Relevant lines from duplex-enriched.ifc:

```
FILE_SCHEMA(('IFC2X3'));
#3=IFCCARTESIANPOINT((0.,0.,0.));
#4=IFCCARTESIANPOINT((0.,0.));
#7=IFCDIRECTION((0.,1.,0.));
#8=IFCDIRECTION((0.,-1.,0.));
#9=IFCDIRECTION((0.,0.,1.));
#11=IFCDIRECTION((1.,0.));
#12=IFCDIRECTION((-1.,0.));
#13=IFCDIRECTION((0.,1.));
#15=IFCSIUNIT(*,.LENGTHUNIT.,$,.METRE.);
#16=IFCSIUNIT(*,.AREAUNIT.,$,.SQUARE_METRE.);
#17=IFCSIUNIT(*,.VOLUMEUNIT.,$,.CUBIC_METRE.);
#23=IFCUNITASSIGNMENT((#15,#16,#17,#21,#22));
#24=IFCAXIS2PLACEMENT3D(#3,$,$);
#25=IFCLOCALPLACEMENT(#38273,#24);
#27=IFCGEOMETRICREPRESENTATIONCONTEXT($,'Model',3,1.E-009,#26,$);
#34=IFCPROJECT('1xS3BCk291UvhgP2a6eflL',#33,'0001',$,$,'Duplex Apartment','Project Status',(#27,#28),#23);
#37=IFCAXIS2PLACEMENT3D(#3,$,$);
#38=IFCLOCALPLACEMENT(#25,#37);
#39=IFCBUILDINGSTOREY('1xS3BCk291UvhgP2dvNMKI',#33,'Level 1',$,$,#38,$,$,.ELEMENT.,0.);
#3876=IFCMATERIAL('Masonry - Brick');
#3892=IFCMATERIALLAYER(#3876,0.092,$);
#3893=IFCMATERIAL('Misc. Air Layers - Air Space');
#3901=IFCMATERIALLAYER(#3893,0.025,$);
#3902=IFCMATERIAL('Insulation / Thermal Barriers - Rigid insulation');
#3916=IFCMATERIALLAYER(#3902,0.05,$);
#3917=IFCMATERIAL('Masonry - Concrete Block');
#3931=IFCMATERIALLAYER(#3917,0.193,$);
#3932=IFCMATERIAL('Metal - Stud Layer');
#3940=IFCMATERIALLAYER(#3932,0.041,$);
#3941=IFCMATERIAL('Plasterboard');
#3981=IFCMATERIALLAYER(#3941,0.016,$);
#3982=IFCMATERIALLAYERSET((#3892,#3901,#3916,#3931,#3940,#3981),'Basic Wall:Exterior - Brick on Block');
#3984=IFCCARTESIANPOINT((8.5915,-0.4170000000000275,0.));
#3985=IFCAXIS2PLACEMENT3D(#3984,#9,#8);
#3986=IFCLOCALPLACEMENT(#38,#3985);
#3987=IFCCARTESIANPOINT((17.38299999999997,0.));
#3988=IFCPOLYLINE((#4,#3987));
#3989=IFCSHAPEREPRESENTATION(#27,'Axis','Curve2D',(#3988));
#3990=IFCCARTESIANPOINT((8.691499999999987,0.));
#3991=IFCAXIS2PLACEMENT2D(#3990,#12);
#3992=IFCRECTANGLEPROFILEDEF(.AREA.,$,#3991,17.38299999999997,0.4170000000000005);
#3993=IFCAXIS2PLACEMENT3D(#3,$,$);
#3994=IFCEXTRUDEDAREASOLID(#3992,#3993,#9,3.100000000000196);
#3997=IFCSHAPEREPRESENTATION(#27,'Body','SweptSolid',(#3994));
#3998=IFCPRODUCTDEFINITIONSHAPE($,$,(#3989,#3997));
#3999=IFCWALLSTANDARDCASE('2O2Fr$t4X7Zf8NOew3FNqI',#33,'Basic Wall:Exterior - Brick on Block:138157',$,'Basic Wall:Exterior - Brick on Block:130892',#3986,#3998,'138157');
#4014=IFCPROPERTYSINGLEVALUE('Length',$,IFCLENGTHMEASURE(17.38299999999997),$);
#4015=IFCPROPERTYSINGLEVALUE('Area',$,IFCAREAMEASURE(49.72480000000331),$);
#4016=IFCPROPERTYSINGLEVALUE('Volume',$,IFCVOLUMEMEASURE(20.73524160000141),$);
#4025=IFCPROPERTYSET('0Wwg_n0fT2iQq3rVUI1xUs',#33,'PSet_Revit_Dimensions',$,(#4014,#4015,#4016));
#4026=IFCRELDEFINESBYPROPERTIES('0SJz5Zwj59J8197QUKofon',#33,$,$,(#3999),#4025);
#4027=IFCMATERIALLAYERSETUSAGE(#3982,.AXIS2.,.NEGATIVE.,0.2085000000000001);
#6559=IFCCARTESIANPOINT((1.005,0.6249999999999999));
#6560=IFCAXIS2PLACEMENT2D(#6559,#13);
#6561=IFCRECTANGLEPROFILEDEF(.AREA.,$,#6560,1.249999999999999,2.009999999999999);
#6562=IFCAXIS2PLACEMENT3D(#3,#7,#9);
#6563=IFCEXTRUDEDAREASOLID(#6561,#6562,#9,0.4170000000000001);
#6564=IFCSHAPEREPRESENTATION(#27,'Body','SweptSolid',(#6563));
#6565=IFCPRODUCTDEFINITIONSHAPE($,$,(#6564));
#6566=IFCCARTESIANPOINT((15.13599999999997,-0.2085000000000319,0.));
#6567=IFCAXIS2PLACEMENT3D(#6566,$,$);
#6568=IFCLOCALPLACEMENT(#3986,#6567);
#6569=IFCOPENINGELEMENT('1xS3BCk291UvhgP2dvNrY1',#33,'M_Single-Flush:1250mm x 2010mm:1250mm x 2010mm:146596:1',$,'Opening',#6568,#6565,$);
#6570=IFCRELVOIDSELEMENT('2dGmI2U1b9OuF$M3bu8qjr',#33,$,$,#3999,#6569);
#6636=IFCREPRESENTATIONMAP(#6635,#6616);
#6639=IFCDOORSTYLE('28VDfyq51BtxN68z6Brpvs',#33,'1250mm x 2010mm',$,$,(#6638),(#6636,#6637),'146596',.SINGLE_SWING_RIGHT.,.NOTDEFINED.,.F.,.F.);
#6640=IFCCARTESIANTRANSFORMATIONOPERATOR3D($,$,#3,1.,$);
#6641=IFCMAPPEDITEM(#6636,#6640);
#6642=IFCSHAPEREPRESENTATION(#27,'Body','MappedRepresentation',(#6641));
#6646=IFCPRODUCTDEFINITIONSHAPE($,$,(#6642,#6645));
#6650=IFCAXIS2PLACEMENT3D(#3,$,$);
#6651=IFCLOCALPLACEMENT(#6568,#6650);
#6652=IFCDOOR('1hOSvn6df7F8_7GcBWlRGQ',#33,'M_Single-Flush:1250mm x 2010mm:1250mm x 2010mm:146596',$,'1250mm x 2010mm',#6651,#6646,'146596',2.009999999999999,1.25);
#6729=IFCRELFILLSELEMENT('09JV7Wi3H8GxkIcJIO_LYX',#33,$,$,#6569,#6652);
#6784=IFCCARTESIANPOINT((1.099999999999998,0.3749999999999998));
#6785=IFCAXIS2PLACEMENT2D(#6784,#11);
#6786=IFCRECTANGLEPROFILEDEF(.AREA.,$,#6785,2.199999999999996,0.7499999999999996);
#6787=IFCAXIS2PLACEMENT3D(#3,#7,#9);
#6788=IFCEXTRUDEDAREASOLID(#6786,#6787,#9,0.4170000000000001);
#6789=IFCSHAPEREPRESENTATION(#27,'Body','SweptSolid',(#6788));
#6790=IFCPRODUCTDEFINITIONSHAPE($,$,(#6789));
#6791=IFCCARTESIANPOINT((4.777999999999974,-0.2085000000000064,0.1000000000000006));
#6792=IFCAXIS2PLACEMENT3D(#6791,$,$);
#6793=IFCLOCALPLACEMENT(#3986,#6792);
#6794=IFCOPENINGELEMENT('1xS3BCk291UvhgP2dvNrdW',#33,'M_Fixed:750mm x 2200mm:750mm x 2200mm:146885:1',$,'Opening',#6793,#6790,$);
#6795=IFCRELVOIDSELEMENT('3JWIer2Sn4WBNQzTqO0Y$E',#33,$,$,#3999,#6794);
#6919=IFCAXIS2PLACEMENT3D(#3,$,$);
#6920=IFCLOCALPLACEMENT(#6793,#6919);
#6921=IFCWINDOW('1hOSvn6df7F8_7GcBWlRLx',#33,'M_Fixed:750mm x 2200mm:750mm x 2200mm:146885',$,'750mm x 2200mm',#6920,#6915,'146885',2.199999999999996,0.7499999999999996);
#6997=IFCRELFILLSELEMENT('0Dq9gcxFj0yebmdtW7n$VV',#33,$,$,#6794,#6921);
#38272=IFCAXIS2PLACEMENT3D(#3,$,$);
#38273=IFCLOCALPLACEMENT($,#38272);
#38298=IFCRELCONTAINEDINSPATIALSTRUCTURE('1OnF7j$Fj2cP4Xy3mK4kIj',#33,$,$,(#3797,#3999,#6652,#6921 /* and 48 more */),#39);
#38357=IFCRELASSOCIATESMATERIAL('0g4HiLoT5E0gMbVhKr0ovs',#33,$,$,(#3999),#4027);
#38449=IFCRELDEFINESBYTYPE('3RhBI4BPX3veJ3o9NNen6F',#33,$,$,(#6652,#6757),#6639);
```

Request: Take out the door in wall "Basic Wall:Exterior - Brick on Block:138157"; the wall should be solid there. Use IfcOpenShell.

```python
import ifcopenshell
import ifcopenshell.api.feature
import ifcopenshell.api.pset
import ifcopenshell.api.root
import ifcopenshell.geom
import ifcopenshell.util.element
import ifcopenshell.util.shape
import ifcopenshell.util.unit

model = ifcopenshell.open("duplex-enriched.ifc")
area_scale = ifcopenshell.util.unit.calculate_unit_scale(model, "AREAUNIT")
volume_scale = ifcopenshell.util.unit.calculate_unit_scale(model, "VOLUMEUNIT")
settings = ifcopenshell.geom.settings()


def volume(element):
    """Net volume in cubic metres, openings subtracted."""
    shape = ifcopenshell.geom.create_shape(settings, element)
    return ifcopenshell.util.shape.get_volume(shape.geometry)


door = model.by_id(6652)
opening = door.FillsVoids[0].RelatingOpeningElement
wall = opening.VoidsElements[0].RelatingBuildingElement
before = volume(wall)

ifcopenshell.api.root.remove_product(model, product=door)
ifcopenshell.api.feature.remove_feature(model, feature=opening)

after = volume(wall)
thickness = 0.417  # wall thickness in metres

# Update the wall's stored quantities.
pset = model.by_id(ifcopenshell.util.element.get_pset(wall, "PSet_Revit_Dimensions", should_inherit=False)["id"])
ifcopenshell.api.pset.edit_pset(model, pset=pset, properties={
    "Area": model.create_entity("IfcAreaMeasure", after / thickness / area_scale),
    "Volume": model.create_entity("IfcVolumeMeasure", after / volume_scale),
})

print(f"wall volume {before:.3f} -> {after:.3f} m3")

model.write("duplex-enriched_updated.ifc")
```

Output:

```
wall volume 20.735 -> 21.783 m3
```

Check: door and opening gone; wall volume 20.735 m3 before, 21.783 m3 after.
